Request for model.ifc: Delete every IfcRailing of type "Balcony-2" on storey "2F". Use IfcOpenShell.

First a look at what the model holds.

```python
import ifcopenshell
import ifcopenshell.util.element

model = ifcopenshell.open("model.ifc")
print(model.schema)
storey = next(s for s in model.by_type("IfcBuildingStorey") if s.Name == "2F")
railings = [e for e in ifcopenshell.util.element.get_decomposition(storey) if e.is_a("IfcRailing")]
seen = {}
for e in railings:
    element_type = ifcopenshell.util.element.get_type(e)
    name = element_type.Name if element_type not in (None, e) else None
    seen[name] = seen.get(name, 0) + 1
for name, count in sorted(seen.items(), key=str):
    print(count, "x", name)
```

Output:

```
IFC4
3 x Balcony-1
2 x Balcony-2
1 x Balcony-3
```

```python
import ifcopenshell
import ifcopenshell.api.root
import ifcopenshell.util.element

model = ifcopenshell.open("model.ifc")

storey = next(s for s in model.by_type("IfcBuildingStorey") if s.Name == "2F")
railings = [e for e in ifcopenshell.util.element.get_decomposition(storey) if e.is_a("IfcRailing")]
targets = [e for e in railings if (t := ifcopenshell.util.element.get_type(e)) not in (None, e) and t.Name == "Balcony-2"]

for e in targets:
    ifcopenshell.api.root.remove_product(model, product=e)
print(len(targets), "removed")

model.write("model-out.ifc")
```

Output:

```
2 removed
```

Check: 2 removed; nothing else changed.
